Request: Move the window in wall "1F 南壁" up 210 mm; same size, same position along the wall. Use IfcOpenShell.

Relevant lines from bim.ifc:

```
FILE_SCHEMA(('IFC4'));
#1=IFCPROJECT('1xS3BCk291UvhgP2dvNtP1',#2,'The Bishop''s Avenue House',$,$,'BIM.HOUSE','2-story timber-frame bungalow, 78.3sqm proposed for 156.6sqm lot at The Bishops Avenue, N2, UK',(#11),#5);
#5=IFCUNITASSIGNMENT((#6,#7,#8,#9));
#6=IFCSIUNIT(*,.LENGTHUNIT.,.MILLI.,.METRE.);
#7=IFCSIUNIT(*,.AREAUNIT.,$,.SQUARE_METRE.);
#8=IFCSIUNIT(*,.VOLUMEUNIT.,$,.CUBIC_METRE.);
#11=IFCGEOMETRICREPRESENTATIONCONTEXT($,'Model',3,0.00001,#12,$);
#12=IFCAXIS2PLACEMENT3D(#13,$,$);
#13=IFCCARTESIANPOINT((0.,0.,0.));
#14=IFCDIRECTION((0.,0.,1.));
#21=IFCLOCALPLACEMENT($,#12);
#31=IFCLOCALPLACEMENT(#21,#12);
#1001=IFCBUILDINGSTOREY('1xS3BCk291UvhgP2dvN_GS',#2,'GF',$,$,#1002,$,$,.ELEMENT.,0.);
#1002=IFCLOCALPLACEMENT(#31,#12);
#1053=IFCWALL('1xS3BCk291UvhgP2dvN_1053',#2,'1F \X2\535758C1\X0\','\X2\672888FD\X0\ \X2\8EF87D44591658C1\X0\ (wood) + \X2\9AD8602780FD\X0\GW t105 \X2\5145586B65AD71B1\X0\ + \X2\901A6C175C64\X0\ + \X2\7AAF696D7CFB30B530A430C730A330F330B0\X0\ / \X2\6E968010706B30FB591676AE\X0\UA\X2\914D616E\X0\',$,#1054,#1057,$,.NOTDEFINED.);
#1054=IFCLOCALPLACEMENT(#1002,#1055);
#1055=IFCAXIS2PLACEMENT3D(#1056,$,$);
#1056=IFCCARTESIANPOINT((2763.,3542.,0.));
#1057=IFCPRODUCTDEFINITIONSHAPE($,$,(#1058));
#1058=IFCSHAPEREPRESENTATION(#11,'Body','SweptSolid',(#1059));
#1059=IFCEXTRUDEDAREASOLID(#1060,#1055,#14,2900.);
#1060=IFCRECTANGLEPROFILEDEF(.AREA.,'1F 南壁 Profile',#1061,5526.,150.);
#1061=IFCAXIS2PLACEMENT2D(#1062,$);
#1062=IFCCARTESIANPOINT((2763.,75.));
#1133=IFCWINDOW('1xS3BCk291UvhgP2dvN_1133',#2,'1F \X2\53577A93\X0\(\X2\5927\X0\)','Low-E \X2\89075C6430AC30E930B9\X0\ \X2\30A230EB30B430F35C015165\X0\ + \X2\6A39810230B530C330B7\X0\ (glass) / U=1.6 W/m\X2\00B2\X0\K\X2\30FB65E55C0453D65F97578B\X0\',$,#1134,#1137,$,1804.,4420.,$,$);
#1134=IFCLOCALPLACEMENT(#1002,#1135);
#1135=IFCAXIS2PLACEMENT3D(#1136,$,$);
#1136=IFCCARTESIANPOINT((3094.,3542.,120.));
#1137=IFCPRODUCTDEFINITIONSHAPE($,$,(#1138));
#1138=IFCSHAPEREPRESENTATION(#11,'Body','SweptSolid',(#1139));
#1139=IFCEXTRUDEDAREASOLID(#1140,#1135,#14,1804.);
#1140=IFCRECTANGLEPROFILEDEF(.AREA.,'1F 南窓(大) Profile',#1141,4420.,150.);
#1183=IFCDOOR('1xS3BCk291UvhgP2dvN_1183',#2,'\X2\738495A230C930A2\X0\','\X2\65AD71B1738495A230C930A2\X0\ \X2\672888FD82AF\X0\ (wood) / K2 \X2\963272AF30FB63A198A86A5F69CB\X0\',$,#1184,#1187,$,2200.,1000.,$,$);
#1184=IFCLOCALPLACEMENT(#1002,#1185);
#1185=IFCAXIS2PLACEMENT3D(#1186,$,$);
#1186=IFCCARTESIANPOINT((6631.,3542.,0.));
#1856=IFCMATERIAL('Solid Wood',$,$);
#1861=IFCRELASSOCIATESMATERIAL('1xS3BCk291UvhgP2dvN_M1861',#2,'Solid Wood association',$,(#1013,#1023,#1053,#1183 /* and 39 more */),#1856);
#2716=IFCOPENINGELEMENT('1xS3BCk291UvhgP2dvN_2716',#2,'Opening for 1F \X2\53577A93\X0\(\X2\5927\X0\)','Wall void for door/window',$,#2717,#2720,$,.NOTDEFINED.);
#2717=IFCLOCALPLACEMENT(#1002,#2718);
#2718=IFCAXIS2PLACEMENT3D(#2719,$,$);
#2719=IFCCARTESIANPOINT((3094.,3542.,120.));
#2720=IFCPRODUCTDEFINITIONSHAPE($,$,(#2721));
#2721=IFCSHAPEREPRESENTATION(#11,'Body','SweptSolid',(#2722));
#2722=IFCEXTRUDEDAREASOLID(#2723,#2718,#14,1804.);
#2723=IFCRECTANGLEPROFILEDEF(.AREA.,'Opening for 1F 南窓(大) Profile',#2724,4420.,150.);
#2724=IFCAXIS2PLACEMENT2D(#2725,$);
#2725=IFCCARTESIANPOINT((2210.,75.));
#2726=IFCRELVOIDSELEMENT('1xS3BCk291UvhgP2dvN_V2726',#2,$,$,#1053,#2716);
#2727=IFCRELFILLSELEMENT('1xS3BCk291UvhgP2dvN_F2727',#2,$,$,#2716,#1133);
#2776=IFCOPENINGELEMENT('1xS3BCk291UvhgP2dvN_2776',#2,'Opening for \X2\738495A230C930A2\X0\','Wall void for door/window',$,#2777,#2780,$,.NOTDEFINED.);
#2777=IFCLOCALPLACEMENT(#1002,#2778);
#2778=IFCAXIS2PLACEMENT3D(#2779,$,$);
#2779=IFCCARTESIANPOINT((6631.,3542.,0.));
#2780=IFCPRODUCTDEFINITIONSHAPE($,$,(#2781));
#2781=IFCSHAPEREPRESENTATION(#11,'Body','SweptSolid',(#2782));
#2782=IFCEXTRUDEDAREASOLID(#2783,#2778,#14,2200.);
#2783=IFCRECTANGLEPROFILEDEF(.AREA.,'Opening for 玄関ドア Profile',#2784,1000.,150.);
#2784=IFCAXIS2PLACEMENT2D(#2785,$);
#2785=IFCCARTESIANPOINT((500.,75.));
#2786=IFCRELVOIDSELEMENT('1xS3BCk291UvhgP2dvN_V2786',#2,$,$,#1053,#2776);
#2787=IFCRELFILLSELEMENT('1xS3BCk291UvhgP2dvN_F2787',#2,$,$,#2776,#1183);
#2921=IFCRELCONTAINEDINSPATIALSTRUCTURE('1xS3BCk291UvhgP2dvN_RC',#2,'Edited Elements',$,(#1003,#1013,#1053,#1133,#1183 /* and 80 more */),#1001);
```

```python
import numpy as np
import ifcopenshell
import ifcopenshell.api.geometry
import ifcopenshell.util.placement
import ifcopenshell.util.unit

model = ifcopenshell.open("bim.ifc")
unit_scale = ifcopenshell.util.unit.calculate_unit_scale(model)

window = model.by_guid("1xS3BCk291UvhgP2dvN_1133")
opening = window.FillsVoids[0].RelatingOpeningElement
dz = 0.21 / unit_scale

shift = np.array([0.0, 0.0, dz])
# The window is not placed relative to its opening, so move both.
for product in (opening, window):
    matrix = ifcopenshell.util.placement.get_local_placement(product.ObjectPlacement)
    matrix[:3, 3] += shift
    ifcopenshell.api.geometry.edit_object_placement(model, product=product, matrix=matrix, is_si=False)

print(f"moved by {dz * unit_scale:+.3f} m")

model.write("bim_v2.ifc")
```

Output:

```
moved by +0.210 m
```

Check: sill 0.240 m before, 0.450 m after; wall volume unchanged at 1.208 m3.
